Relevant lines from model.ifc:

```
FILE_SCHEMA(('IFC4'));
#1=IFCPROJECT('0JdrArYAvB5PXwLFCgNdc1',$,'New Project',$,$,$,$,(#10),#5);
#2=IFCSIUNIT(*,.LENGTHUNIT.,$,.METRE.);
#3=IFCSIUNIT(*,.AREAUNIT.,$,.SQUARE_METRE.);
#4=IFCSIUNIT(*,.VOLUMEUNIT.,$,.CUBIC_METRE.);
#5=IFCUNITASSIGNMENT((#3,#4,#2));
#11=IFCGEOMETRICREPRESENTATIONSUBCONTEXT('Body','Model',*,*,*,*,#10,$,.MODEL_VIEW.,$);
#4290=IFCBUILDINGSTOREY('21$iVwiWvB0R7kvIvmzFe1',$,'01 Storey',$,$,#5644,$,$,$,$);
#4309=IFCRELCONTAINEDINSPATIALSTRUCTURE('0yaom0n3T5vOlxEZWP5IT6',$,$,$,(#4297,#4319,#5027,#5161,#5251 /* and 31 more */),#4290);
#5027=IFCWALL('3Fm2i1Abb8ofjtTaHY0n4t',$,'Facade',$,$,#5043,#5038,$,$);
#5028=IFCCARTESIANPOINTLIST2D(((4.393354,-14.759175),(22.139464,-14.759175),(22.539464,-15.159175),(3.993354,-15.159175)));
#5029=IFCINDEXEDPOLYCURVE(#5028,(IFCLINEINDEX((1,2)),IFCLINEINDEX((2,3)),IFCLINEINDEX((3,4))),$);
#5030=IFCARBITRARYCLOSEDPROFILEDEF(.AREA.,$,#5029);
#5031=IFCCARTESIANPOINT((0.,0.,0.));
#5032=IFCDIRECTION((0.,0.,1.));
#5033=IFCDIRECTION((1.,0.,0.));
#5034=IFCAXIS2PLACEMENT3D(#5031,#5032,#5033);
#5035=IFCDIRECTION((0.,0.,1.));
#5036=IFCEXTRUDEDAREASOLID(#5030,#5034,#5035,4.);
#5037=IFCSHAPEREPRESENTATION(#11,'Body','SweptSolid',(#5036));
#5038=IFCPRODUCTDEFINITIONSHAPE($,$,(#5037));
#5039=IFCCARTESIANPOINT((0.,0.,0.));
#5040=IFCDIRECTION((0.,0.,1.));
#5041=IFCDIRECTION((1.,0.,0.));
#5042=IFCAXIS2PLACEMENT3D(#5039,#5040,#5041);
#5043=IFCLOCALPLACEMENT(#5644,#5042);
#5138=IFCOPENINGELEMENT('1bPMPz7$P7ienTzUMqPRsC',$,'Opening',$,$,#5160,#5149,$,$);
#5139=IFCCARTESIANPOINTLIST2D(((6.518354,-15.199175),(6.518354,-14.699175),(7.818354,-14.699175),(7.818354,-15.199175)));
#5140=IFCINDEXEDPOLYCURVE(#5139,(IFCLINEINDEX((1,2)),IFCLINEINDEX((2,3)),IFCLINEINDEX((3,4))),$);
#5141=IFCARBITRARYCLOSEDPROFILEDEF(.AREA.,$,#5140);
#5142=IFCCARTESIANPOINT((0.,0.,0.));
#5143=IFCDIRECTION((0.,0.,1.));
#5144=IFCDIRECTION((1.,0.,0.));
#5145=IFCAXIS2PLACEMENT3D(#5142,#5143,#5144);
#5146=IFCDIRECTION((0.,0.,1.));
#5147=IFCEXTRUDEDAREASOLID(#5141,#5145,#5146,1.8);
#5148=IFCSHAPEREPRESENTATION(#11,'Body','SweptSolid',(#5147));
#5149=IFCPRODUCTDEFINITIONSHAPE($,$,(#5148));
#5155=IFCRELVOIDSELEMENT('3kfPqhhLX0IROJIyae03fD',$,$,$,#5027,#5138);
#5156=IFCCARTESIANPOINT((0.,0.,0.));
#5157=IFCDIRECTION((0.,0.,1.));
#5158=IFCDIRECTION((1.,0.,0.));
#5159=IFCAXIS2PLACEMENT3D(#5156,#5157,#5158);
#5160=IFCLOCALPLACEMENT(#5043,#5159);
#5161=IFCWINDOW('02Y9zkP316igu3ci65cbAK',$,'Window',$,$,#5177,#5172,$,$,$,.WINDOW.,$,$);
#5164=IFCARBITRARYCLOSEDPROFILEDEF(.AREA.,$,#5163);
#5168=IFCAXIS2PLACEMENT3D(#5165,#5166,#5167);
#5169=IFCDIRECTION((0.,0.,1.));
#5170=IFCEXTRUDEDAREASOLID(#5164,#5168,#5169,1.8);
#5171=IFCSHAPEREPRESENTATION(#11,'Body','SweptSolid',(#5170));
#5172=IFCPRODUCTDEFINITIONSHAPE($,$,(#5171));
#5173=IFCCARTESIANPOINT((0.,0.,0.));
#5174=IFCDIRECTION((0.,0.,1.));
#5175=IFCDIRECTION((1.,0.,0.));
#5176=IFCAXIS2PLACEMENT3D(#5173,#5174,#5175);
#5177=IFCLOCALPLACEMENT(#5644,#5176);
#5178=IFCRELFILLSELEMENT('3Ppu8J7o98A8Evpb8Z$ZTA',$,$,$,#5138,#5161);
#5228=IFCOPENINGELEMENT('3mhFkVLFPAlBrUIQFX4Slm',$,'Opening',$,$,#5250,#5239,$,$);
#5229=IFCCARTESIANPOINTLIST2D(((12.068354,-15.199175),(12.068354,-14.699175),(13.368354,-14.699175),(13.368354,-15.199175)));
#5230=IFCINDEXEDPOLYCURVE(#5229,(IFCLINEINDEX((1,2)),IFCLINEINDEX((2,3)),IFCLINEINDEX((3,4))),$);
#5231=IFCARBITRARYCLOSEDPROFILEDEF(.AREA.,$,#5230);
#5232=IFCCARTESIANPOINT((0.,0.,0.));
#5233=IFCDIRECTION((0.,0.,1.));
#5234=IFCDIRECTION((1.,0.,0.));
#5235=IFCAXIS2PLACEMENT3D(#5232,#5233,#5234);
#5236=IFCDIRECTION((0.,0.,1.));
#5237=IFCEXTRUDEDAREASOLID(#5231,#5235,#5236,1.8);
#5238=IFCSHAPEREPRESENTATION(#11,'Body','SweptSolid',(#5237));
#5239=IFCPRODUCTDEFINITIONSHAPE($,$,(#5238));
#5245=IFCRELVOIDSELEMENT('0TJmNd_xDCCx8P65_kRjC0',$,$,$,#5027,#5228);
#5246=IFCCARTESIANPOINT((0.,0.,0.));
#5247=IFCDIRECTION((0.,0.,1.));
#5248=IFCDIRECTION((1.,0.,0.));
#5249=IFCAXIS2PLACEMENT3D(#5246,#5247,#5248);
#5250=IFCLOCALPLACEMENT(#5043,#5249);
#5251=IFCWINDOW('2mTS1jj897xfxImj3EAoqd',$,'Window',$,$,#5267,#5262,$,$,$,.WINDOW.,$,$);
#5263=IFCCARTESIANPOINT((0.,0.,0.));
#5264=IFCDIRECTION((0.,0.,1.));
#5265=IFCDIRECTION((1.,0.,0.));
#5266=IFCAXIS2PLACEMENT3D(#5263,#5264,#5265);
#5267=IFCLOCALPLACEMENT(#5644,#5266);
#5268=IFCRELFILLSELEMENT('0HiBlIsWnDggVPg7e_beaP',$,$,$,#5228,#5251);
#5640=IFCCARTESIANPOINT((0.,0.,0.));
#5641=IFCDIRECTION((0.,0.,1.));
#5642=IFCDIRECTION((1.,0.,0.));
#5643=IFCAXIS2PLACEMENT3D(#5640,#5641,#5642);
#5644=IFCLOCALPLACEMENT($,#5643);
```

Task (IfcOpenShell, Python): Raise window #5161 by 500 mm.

```python
import numpy as np
import ifcopenshell
import ifcopenshell.api.geometry
import ifcopenshell.util.placement
import ifcopenshell.util.unit

model = ifcopenshell.open("model.ifc")
unit_scale = ifcopenshell.util.unit.calculate_unit_scale(model)

window = model.by_guid("02Y9zkP316igu3ci65cbAK")
opening = window.FillsVoids[0].RelatingOpeningElement
dz = 0.5 / unit_scale

shift = np.array([0.0, 0.0, dz])
# The window is not placed relative to its opening, so move both.
for product in (opening, window):
    matrix = ifcopenshell.util.placement.get_local_placement(product.ObjectPlacement)
    matrix[:3, 3] += shift
    ifcopenshell.api.geometry.edit_object_placement(model, product=product, matrix=matrix, is_si=False)

print(f"moved by {dz * unit_scale:+.3f} m")

model.write("model_rev.ifc")
```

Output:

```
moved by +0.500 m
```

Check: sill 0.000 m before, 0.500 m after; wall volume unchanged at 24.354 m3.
